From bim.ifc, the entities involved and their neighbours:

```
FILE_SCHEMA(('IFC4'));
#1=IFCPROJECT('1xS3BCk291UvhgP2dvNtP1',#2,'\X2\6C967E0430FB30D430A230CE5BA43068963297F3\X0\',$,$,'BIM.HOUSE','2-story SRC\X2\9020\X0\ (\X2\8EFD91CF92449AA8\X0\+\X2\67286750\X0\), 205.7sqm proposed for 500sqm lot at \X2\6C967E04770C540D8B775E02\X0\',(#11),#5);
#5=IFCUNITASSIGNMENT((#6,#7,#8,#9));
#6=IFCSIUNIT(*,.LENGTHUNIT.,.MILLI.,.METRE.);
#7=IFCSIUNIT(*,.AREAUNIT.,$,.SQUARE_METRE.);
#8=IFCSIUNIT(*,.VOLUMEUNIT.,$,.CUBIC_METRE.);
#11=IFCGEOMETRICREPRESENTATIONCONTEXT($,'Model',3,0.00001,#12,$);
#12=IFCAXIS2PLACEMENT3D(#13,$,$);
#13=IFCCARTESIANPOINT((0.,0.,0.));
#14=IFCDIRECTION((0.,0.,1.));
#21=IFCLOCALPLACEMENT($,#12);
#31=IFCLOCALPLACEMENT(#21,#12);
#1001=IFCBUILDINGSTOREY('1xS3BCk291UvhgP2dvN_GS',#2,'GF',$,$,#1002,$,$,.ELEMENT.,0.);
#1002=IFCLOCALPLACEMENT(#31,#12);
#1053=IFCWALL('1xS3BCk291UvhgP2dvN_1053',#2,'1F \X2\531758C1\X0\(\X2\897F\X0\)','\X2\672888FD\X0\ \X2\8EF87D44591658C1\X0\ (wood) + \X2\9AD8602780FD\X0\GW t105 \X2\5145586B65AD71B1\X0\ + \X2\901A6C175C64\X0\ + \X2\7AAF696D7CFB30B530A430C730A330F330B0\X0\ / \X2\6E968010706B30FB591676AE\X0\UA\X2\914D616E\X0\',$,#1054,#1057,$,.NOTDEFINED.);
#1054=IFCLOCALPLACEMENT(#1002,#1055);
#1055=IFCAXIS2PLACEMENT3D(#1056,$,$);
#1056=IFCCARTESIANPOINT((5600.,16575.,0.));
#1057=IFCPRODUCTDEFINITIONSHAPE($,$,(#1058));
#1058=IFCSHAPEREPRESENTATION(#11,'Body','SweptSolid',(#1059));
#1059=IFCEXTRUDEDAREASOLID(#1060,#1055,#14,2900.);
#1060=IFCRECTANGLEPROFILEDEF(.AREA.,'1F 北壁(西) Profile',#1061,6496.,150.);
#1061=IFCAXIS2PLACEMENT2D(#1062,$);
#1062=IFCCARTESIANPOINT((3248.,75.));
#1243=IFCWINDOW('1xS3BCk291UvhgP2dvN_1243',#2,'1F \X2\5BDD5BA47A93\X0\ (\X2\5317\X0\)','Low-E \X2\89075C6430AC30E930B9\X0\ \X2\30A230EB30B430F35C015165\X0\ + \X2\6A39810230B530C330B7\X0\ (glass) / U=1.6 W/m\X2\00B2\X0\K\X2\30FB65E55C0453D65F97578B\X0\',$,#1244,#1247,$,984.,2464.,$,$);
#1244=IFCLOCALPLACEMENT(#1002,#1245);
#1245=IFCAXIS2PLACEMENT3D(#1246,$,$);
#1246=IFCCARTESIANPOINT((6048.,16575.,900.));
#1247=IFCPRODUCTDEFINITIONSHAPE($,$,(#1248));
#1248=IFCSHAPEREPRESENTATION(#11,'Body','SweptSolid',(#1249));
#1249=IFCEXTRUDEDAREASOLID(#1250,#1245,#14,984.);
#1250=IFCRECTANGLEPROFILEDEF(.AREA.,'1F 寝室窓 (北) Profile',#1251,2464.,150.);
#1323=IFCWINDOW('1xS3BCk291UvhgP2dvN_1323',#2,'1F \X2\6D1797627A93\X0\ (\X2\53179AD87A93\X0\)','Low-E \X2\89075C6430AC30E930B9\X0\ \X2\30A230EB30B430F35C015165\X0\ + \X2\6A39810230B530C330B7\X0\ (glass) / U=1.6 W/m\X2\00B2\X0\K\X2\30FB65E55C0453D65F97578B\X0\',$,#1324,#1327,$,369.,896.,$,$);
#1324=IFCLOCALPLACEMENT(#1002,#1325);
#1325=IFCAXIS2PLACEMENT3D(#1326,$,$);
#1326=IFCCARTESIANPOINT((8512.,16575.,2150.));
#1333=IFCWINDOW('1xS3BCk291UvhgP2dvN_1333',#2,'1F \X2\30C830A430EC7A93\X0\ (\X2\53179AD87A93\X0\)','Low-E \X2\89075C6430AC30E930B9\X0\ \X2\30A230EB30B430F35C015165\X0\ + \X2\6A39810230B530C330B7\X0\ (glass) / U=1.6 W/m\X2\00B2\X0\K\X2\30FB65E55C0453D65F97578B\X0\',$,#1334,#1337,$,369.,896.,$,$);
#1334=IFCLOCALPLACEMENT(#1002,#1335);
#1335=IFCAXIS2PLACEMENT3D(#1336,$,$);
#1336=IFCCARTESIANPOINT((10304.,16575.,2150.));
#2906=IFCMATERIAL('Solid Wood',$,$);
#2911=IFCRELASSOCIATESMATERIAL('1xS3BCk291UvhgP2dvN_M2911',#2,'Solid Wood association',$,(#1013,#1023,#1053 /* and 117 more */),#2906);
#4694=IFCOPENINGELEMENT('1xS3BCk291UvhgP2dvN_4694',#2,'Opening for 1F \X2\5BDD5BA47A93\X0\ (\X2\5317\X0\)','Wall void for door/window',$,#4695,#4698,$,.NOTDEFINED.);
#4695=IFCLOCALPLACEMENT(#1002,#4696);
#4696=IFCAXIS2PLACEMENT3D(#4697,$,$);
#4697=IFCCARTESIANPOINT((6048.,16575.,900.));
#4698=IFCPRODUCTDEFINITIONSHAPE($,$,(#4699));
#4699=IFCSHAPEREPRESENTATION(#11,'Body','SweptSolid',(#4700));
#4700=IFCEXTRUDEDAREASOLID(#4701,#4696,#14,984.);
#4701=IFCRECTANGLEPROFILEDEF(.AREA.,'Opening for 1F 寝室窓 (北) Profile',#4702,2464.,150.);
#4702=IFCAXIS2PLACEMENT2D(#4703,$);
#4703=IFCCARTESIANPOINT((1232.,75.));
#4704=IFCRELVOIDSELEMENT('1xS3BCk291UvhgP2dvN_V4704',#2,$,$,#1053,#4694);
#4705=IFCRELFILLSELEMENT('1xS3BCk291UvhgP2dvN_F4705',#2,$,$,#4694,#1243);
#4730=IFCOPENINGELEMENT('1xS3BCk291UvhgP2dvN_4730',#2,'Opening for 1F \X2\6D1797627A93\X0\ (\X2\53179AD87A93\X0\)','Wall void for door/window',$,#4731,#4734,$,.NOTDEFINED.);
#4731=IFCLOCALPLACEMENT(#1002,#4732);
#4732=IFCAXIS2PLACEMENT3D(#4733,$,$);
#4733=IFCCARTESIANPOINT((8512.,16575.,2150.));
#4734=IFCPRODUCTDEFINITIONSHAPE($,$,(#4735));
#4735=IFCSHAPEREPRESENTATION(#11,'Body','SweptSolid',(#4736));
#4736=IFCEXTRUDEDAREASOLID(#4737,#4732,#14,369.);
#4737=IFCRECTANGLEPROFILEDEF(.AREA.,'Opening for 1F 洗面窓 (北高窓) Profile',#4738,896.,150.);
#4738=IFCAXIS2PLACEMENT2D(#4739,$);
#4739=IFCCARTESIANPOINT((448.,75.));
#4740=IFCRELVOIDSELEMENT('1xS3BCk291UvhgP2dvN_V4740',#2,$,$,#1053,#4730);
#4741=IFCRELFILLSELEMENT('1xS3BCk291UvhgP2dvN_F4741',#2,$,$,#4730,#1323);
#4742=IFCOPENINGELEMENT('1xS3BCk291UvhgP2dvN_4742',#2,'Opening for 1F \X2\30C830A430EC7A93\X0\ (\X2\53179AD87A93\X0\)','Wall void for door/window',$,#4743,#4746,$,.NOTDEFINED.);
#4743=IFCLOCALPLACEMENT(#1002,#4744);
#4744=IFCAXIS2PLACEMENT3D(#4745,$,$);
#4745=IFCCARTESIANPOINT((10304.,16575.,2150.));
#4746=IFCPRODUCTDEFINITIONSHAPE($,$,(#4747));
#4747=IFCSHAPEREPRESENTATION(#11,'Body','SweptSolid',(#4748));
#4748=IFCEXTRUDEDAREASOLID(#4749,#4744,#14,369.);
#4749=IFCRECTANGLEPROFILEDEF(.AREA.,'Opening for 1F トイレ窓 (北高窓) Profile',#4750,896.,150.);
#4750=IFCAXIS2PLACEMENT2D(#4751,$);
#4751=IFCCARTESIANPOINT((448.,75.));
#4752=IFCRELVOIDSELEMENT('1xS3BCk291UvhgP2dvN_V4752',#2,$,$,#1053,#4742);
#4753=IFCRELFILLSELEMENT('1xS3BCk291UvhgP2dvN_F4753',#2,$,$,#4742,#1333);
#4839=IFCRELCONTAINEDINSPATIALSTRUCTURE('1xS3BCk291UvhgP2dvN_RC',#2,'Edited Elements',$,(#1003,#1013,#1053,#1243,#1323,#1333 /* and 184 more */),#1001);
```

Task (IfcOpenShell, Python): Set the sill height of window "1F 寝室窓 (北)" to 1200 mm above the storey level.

```python
import numpy as np
import ifcopenshell
import ifcopenshell.api.geometry
import ifcopenshell.geom
import ifcopenshell.util.element
import ifcopenshell.util.placement
import ifcopenshell.util.shape
import ifcopenshell.util.unit

model = ifcopenshell.open("bim.ifc")
unit_scale = ifcopenshell.util.unit.calculate_unit_scale(model)

window = model.by_guid("1xS3BCk291UvhgP2dvN_1243")
opening = window.FillsVoids[0].RelatingOpeningElement
storey = ifcopenshell.util.element.get_container(window, ifc_class="IfcBuildingStorey")
level = ifcopenshell.util.placement.get_local_placement(storey.ObjectPlacement)[2, 3]

# The opening's origin need not be at the sill, so measure its lowest point.
shape = ifcopenshell.geom.create_shape(ifcopenshell.geom.settings(), opening)
bottom = ifcopenshell.util.shape.get_shape_bottom_elevation(shape, shape.geometry) / unit_scale
dz = level + 1200.0 - bottom

shift = np.array([0.0, 0.0, dz])
# The window is not placed relative to its opening, so move both.
for product in (opening, window):
    matrix = ifcopenshell.util.placement.get_local_placement(product.ObjectPlacement)
    matrix[:3, 3] += shift
    ifcopenshell.api.geometry.edit_object_placement(model, product=product, matrix=matrix, is_si=False)

print(f"moved by {dz * unit_scale:+.3f} m")

model.write("bim_updated.ifc")
```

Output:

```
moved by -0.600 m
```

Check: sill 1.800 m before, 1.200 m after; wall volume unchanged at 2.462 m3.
